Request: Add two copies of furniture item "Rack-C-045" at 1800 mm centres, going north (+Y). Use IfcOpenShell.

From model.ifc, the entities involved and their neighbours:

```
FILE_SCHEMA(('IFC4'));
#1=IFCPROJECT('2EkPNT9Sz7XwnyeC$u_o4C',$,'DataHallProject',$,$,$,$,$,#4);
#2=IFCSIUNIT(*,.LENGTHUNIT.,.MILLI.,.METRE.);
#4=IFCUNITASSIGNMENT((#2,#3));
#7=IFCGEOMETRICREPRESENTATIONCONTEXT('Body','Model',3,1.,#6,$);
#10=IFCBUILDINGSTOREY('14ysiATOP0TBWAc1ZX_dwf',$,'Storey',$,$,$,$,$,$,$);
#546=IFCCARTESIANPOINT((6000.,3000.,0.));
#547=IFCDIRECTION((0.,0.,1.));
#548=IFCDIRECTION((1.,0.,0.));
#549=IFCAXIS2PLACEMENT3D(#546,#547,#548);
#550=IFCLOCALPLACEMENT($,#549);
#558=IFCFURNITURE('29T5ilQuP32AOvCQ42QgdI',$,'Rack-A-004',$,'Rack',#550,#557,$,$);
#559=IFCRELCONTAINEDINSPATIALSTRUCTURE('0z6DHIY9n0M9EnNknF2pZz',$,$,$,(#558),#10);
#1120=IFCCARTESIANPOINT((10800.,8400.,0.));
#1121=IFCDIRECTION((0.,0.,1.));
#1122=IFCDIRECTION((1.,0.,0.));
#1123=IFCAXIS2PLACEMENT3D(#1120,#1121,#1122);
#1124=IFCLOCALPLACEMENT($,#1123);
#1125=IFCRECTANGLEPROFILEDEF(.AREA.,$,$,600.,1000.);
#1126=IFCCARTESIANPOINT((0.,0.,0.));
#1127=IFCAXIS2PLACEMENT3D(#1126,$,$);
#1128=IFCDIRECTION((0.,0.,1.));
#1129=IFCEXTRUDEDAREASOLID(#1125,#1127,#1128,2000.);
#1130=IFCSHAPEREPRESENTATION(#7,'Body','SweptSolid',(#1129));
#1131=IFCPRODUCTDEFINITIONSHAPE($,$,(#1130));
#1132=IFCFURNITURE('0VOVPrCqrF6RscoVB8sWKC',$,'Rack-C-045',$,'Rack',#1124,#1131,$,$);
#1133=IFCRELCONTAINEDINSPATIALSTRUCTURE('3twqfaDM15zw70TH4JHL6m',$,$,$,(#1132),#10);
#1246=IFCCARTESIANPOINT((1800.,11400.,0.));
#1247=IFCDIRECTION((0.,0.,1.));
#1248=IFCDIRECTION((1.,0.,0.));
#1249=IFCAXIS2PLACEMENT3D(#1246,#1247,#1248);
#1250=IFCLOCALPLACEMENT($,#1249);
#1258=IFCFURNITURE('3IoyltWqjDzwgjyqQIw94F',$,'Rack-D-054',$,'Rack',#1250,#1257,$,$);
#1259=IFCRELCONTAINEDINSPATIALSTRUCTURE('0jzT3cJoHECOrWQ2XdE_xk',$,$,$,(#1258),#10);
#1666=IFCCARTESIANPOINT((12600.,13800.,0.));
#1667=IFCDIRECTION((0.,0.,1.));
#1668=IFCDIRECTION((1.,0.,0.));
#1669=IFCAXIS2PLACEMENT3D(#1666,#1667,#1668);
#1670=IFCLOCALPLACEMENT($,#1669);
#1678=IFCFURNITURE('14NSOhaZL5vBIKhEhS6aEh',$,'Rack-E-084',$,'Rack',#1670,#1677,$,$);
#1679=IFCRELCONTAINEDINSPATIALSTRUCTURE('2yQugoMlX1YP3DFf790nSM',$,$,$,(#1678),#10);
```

```python
import numpy as np
import ifcopenshell
import ifcopenshell.api.geometry
import ifcopenshell.api.root
import ifcopenshell.util.element
import ifcopenshell.util.placement
import ifcopenshell.util.unit

model = ifcopenshell.open("model.ifc")
unit_scale = ifcopenshell.util.unit.calculate_unit_scale(model)

source = model.by_guid("0VOVPrCqrF6RscoVB8sWKC")
base = ifcopenshell.util.placement.get_local_placement(source.ObjectPlacement)
step = np.array([0.0, 1.0, 0.0]) * 1.8 / unit_scale

for i in range(1, 3):
    copy = ifcopenshell.api.root.copy_class(model, product=source)
    copy.Representation = ifcopenshell.util.element.copy_deep(
        model, source.Representation, exclude=["IfcGeometricRepresentationContext", "IfcRepresentationMap"]
    )
    matrix = base.copy()
    matrix[:3, 3] += i * step
    print("added at", matrix[:3, 3].round(3) + 0.0)
    ifcopenshell.api.geometry.edit_object_placement(model, product=copy, matrix=matrix, is_si=False)

model.write("model_v2.ifc")
```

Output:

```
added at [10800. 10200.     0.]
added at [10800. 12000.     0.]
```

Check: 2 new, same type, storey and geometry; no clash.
